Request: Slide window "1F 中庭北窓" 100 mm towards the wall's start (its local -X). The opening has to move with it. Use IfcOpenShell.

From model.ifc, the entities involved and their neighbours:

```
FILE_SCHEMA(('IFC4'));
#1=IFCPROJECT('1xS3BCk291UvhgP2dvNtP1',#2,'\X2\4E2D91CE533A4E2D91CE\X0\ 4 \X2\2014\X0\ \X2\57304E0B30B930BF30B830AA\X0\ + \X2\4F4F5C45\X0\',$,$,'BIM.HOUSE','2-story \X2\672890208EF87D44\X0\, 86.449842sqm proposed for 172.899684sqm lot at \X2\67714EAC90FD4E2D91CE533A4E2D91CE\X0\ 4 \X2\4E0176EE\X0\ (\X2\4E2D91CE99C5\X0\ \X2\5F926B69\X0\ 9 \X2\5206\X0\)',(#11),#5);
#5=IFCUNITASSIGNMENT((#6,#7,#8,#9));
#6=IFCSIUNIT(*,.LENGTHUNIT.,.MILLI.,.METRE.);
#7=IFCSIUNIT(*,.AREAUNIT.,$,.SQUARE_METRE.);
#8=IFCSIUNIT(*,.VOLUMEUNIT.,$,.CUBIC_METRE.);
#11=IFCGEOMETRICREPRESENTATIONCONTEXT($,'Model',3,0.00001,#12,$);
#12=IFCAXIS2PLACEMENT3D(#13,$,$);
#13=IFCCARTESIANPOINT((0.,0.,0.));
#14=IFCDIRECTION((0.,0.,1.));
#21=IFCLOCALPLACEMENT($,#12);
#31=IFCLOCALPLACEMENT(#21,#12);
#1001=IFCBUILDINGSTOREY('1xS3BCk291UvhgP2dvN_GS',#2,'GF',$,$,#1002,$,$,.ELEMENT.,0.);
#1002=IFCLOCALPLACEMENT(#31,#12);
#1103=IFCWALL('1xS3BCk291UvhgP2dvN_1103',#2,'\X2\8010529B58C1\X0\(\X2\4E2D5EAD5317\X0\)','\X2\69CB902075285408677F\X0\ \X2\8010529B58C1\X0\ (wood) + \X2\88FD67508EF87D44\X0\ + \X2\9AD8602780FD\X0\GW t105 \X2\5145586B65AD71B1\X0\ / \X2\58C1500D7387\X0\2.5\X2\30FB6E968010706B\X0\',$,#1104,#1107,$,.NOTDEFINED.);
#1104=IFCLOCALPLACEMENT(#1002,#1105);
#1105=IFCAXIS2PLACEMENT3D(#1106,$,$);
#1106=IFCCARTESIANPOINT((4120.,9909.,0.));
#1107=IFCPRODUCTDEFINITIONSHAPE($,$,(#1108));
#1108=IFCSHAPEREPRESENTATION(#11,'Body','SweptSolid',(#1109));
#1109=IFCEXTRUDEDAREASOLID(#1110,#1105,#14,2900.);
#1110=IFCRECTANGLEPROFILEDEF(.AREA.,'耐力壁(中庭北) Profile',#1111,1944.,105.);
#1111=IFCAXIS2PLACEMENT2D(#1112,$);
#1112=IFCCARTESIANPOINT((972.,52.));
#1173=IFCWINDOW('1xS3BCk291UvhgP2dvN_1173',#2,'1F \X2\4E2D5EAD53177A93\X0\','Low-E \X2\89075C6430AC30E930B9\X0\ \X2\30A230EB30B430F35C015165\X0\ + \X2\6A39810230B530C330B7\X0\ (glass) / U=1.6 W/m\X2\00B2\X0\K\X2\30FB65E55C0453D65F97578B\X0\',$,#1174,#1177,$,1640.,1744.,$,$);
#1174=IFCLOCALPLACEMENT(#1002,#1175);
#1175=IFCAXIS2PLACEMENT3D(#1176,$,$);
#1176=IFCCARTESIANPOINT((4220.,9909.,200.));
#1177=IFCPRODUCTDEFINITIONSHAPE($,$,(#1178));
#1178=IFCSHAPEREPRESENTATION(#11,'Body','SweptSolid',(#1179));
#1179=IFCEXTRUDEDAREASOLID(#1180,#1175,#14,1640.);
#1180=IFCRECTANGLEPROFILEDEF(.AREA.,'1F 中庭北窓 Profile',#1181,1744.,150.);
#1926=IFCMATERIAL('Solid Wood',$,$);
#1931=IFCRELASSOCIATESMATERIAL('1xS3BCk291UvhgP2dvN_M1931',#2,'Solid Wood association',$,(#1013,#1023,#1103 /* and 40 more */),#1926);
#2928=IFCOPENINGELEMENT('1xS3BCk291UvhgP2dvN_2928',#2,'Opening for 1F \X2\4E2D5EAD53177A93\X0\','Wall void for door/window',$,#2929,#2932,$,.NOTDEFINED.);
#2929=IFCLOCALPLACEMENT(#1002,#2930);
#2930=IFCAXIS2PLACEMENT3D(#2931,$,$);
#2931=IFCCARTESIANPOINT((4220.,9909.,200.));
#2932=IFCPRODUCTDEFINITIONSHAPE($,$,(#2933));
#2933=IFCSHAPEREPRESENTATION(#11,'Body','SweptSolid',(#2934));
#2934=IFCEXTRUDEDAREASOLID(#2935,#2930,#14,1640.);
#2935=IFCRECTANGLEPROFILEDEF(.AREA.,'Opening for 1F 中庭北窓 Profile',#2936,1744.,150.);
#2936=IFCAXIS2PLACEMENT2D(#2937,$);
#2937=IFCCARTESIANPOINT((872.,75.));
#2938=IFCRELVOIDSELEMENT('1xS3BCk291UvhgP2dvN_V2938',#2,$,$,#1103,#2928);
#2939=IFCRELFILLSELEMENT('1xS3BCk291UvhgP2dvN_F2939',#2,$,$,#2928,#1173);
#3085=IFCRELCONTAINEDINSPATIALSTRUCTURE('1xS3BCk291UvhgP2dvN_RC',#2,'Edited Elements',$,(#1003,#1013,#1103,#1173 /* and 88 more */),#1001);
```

```python
import ifcopenshell
import ifcopenshell.api.geometry
import ifcopenshell.util.placement
import ifcopenshell.util.unit

model = ifcopenshell.open("model.ifc")
unit_scale = ifcopenshell.util.unit.calculate_unit_scale(model)

window = model.by_guid("1xS3BCk291UvhgP2dvN_1173")
opening = window.FillsVoids[0].RelatingOpeningElement
wall = opening.VoidsElements[0].RelatingBuildingElement

wall_matrix = ifcopenshell.util.placement.get_local_placement(wall.ObjectPlacement)
shift = wall_matrix[:3, 0] * -0.1 / unit_scale
before = ifcopenshell.util.placement.get_local_placement(window.ObjectPlacement)[:3, 3].copy()

# The window is not placed relative to its opening, so move both.
for product in (opening, window):
    matrix = ifcopenshell.util.placement.get_local_placement(product.ObjectPlacement)
    matrix[:3, 3] += shift
    ifcopenshell.api.geometry.edit_object_placement(model, product=product, matrix=matrix, is_si=False)

after = ifcopenshell.util.placement.get_local_placement(window.ObjectPlacement)[:3, 3]
print("window moved by", (after - before).round(3) + 0.0)

model.write("model_v2.ifc")
```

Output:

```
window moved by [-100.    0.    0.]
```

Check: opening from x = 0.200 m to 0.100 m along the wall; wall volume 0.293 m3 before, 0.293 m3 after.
